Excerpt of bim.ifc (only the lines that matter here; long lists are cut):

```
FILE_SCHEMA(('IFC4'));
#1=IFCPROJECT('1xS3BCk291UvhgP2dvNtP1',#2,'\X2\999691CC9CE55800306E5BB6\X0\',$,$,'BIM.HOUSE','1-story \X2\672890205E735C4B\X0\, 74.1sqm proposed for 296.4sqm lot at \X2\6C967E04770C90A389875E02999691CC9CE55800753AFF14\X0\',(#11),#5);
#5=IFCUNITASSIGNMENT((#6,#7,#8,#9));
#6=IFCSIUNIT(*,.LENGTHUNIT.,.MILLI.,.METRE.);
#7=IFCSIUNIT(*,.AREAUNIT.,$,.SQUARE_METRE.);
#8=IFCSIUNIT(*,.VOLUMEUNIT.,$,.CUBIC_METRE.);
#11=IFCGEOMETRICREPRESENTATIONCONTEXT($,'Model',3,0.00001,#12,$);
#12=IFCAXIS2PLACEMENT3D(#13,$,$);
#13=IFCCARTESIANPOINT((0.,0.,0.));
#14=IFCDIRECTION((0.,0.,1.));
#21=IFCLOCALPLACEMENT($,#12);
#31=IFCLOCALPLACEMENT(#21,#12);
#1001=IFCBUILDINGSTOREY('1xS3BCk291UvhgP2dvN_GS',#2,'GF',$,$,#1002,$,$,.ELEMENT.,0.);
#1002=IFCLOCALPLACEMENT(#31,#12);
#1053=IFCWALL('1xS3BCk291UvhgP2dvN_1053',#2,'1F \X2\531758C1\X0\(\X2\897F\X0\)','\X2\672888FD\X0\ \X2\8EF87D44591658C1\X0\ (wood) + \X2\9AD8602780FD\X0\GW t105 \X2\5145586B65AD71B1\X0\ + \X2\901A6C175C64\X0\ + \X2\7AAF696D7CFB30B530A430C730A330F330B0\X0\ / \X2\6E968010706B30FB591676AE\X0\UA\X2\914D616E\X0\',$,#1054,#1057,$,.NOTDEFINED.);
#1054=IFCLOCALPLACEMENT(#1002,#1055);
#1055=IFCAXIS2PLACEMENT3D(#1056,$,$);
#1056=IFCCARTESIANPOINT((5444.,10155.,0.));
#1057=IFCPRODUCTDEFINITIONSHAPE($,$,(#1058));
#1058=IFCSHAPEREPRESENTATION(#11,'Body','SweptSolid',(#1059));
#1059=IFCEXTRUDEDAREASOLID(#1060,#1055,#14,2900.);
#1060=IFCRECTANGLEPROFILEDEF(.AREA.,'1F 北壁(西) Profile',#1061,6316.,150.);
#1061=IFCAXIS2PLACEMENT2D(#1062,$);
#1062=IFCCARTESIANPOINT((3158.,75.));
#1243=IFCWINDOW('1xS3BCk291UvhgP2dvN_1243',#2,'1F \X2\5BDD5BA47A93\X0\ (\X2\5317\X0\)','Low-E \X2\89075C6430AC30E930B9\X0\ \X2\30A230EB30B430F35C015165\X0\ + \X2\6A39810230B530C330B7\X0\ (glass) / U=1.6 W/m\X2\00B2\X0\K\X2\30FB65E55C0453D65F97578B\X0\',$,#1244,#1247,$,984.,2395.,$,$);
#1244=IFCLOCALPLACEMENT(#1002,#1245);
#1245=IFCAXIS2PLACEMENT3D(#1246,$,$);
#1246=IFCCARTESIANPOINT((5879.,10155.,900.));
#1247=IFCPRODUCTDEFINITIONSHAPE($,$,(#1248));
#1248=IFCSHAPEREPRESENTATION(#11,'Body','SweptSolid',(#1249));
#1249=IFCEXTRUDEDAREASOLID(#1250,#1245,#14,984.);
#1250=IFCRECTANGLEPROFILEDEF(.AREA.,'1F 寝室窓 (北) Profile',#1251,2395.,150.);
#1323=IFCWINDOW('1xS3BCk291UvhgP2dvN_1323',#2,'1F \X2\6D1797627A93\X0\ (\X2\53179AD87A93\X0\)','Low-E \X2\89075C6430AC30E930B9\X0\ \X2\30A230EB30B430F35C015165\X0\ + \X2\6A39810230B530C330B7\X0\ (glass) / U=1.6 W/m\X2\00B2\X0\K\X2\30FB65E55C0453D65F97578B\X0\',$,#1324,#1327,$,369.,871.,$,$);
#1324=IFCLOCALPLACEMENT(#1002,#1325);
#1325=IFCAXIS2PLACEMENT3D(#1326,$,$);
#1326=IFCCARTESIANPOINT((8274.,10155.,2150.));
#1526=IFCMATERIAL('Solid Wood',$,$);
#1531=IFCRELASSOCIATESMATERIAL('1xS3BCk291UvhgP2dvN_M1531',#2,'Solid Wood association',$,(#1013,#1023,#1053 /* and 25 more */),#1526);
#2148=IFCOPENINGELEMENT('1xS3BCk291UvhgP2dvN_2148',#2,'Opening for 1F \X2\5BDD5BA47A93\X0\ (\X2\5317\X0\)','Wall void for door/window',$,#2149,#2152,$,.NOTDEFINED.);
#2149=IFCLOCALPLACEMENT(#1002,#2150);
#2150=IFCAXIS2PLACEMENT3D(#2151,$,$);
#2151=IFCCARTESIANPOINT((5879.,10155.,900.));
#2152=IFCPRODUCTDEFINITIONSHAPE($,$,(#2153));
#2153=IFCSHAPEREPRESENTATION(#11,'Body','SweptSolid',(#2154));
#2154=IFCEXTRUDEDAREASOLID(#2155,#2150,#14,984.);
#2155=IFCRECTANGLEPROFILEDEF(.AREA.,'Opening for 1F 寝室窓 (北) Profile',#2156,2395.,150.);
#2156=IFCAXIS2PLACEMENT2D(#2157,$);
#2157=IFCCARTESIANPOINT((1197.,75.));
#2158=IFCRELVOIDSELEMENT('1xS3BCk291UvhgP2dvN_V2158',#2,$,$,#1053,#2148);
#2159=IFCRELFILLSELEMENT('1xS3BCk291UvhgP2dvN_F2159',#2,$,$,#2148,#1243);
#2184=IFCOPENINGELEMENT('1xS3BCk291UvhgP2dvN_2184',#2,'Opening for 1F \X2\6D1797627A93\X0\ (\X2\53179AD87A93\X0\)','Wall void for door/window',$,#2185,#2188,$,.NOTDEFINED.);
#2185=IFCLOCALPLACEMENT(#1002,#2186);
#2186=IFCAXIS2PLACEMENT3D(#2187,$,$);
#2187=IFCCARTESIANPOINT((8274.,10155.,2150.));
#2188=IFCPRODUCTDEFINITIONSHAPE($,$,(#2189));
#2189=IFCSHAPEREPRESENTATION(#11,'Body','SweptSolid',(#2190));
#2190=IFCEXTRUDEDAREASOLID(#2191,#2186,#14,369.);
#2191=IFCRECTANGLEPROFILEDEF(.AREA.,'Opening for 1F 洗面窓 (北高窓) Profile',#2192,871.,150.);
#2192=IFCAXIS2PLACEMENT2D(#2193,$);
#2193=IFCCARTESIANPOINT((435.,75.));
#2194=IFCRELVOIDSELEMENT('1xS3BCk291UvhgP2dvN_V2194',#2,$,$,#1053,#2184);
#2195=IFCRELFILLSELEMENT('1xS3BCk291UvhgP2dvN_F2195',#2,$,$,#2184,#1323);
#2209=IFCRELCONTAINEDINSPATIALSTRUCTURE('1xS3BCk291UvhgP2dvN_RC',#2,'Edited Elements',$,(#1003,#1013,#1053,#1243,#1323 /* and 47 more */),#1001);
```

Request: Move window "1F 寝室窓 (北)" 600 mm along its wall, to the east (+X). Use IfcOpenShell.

```python
import ifcopenshell
import ifcopenshell.api.geometry
import ifcopenshell.util.placement
import ifcopenshell.util.unit

model = ifcopenshell.open("bim.ifc")
unit_scale = ifcopenshell.util.unit.calculate_unit_scale(model)

window = model.by_id(1243)
opening = window.FillsVoids[0].RelatingOpeningElement
wall = opening.VoidsElements[0].RelatingBuildingElement

wall_matrix = ifcopenshell.util.placement.get_local_placement(wall.ObjectPlacement)
shift = wall_matrix[:3, 0] * 0.6 / unit_scale
before = ifcopenshell.util.placement.get_local_placement(window.ObjectPlacement)[:3, 3].copy()

# The window is not placed relative to its opening, so move both.
for product in (opening, window):
    matrix = ifcopenshell.util.placement.get_local_placement(product.ObjectPlacement)
    matrix[:3, 3] += shift
    ifcopenshell.api.geometry.edit_object_placement(model, product=product, matrix=matrix, is_si=False)

after = ifcopenshell.util.placement.get_local_placement(window.ObjectPlacement)[:3, 3]
print("window moved by", (after - before).round(3) + 0.0)

model.write("bim_v2.ifc")
```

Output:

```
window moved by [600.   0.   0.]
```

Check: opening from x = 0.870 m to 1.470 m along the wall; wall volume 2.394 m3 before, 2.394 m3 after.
